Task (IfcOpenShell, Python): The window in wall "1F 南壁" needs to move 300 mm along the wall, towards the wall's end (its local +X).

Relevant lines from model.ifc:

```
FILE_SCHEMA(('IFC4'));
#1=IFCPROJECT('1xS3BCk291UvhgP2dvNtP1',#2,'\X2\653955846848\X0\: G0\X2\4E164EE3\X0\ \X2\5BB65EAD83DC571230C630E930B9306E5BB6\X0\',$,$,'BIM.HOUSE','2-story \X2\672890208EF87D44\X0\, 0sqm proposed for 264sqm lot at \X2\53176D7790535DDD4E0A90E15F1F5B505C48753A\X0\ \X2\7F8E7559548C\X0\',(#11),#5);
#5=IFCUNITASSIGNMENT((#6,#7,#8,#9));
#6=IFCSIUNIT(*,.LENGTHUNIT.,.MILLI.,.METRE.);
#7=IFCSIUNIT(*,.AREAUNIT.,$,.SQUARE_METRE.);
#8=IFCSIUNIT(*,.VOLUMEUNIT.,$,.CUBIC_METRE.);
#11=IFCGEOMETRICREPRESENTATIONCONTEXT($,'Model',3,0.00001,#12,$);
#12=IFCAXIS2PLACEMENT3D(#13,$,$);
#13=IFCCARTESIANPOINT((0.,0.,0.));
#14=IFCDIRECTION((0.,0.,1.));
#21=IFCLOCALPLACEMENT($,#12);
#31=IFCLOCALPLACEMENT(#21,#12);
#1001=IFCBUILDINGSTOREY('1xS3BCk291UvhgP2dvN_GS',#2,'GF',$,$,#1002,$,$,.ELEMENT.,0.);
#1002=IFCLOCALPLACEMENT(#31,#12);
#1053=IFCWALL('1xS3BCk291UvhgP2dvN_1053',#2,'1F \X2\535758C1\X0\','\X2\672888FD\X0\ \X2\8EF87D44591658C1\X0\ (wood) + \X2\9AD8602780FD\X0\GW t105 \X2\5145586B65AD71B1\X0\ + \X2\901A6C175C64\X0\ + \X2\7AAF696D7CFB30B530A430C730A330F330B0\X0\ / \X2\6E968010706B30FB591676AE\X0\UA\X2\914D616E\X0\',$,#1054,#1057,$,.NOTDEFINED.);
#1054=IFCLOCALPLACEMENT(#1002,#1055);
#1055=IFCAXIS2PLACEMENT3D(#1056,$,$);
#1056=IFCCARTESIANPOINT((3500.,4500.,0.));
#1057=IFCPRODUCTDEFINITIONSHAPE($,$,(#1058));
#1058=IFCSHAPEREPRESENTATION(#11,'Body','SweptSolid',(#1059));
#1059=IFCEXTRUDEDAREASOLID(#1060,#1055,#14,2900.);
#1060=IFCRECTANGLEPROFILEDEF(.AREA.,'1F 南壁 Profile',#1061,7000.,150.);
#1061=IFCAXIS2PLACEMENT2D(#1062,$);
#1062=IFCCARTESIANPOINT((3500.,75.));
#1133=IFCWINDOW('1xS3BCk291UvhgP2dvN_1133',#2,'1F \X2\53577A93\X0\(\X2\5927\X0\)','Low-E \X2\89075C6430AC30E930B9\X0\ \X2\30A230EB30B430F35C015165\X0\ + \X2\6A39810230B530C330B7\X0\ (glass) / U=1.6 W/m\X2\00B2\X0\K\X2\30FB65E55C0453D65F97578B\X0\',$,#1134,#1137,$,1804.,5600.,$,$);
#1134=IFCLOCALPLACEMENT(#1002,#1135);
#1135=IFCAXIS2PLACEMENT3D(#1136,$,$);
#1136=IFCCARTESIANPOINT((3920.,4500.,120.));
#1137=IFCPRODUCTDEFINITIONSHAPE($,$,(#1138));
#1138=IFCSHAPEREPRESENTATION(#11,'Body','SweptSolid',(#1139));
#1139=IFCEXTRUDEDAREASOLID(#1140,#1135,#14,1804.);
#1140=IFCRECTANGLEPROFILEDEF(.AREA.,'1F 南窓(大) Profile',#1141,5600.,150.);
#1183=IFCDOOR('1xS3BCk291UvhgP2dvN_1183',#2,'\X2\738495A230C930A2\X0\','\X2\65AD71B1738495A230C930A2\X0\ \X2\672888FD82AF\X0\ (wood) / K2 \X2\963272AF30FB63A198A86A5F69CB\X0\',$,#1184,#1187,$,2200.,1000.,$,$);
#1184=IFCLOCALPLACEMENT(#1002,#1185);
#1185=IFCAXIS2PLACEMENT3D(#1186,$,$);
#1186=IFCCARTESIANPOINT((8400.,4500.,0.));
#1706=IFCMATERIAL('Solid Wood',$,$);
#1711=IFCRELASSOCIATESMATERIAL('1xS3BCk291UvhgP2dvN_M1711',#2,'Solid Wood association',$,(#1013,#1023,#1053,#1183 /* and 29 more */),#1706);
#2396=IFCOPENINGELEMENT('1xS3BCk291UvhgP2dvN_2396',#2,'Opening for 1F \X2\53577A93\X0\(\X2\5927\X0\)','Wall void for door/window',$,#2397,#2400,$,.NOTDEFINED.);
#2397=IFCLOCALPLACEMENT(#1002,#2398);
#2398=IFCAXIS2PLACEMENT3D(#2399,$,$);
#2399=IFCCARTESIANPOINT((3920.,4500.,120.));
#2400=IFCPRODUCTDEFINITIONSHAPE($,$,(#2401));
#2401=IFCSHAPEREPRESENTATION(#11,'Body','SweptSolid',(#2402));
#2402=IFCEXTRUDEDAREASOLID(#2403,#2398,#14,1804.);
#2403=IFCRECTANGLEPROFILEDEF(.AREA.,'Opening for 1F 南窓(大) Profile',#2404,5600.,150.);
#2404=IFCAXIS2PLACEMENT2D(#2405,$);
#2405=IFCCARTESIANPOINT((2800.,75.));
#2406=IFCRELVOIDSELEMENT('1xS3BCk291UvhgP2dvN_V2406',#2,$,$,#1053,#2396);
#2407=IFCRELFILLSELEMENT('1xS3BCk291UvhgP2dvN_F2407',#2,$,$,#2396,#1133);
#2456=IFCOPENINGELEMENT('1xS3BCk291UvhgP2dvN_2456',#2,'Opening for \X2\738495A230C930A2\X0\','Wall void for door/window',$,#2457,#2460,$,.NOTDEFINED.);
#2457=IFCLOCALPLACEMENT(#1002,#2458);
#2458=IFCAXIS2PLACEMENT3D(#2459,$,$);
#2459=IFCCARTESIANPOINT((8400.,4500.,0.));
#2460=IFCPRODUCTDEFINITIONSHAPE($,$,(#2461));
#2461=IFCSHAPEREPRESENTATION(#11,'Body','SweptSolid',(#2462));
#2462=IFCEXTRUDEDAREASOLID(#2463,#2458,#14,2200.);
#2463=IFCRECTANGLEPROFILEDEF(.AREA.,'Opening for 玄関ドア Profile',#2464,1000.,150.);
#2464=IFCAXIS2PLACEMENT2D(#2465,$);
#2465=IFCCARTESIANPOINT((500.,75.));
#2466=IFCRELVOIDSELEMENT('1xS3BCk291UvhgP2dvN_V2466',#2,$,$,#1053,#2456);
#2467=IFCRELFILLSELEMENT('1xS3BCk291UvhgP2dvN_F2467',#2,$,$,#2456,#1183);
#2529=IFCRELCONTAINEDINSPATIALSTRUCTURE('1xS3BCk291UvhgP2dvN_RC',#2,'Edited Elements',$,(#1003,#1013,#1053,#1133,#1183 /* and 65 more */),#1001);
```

```python
import ifcopenshell
import ifcopenshell.api.geometry
import ifcopenshell.util.placement
import ifcopenshell.util.unit

model = ifcopenshell.open("model.ifc")
unit_scale = ifcopenshell.util.unit.calculate_unit_scale(model)

window = model.by_guid("1xS3BCk291UvhgP2dvN_1133")
opening = window.FillsVoids[0].RelatingOpeningElement
wall = opening.VoidsElements[0].RelatingBuildingElement

wall_matrix = ifcopenshell.util.placement.get_local_placement(wall.ObjectPlacement)
shift = wall_matrix[:3, 0] * 0.3 / unit_scale
before = ifcopenshell.util.placement.get_local_placement(window.ObjectPlacement)[:3, 3].copy()

# The window is not placed relative to its opening, so move both.
for product in (opening, window):
    matrix = ifcopenshell.util.placement.get_local_placement(product.ObjectPlacement)
    matrix[:3, 3] += shift
    ifcopenshell.api.geometry.edit_object_placement(model, product=product, matrix=matrix, is_si=False)

after = ifcopenshell.util.placement.get_local_placement(window.ObjectPlacement)[:3, 3]
print("window moved by", (after - before).round(3) + 0.0)

model.write("model-out.ifc")
```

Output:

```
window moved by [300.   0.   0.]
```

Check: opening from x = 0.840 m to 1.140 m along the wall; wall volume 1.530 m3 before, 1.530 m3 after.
